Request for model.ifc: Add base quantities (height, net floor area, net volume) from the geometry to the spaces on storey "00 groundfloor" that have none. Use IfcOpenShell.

First a look at what the model holds.

```python
import ifcopenshell
import ifcopenshell.util.element
import ifcopenshell.util.unit

model = ifcopenshell.open("model.ifc")
print(model.schema)
for unit_type in ("LENGTHUNIT", "AREAUNIT", "VOLUMEUNIT"):
    print(unit_type, ifcopenshell.util.unit.calculate_unit_scale(model, unit_type))
storey = next(s for s in model.by_type("IfcBuildingStorey") if s.Name == "00 groundfloor")
spaces = [e for e in ifcopenshell.util.element.get_decomposition(storey) if e.is_a("IfcSpace")]
for e in sorted(spaces, key=lambda e: e.id()):
    print(e.id(), e.is_a(), e.Name, list(ifcopenshell.util.element.get_psets(e, qtos_only=True)), sep=" | ")
```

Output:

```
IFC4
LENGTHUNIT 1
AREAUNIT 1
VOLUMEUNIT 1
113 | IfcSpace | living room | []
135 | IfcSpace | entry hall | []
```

```python
import ifcopenshell
import ifcopenshell.api.pset
import ifcopenshell.geom
import ifcopenshell.util.element
import ifcopenshell.util.shape
import ifcopenshell.util.unit

model = ifcopenshell.open("model.ifc")
unit_scale = ifcopenshell.util.unit.calculate_unit_scale(model)
area_scale = ifcopenshell.util.unit.calculate_unit_scale(model, "AREAUNIT")
volume_scale = ifcopenshell.util.unit.calculate_unit_scale(model, "VOLUMEUNIT")
settings = ifcopenshell.geom.settings()

storey = next(s for s in model.by_type("IfcBuildingStorey") if s.Name == "00 groundfloor")
spaces = [e for e in ifcopenshell.util.element.get_decomposition(storey) if e.is_a("IfcSpace")]

for e in sorted(spaces, key=lambda e: e.id()):
    if ifcopenshell.util.element.get_psets(e, qtos_only=True, should_inherit=False):
        continue
    # Geometry comes back in metres, in the element's own axes.
    shape = ifcopenshell.geom.create_shape(settings, e)
    values = {
        "Height": ifcopenshell.util.shape.get_z(shape.geometry) / unit_scale,
        "NetFloorArea": ifcopenshell.util.shape.get_footprint_area(shape.geometry) / area_scale,
        "NetVolume": ifcopenshell.util.shape.get_volume(shape.geometry) / volume_scale,
    }
    qto = ifcopenshell.api.pset.add_qto(model, product=e, name="Qto_SpaceBaseQuantities")
    ifcopenshell.api.pset.edit_qto(model, qto=qto, properties=values)
    print(e.id(), {k: round(v, 3) for k, v in values.items()})

model.write("model_edited.ifc")
```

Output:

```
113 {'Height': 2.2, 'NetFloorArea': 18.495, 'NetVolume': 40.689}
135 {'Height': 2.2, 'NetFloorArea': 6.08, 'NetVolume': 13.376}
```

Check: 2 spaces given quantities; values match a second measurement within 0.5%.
